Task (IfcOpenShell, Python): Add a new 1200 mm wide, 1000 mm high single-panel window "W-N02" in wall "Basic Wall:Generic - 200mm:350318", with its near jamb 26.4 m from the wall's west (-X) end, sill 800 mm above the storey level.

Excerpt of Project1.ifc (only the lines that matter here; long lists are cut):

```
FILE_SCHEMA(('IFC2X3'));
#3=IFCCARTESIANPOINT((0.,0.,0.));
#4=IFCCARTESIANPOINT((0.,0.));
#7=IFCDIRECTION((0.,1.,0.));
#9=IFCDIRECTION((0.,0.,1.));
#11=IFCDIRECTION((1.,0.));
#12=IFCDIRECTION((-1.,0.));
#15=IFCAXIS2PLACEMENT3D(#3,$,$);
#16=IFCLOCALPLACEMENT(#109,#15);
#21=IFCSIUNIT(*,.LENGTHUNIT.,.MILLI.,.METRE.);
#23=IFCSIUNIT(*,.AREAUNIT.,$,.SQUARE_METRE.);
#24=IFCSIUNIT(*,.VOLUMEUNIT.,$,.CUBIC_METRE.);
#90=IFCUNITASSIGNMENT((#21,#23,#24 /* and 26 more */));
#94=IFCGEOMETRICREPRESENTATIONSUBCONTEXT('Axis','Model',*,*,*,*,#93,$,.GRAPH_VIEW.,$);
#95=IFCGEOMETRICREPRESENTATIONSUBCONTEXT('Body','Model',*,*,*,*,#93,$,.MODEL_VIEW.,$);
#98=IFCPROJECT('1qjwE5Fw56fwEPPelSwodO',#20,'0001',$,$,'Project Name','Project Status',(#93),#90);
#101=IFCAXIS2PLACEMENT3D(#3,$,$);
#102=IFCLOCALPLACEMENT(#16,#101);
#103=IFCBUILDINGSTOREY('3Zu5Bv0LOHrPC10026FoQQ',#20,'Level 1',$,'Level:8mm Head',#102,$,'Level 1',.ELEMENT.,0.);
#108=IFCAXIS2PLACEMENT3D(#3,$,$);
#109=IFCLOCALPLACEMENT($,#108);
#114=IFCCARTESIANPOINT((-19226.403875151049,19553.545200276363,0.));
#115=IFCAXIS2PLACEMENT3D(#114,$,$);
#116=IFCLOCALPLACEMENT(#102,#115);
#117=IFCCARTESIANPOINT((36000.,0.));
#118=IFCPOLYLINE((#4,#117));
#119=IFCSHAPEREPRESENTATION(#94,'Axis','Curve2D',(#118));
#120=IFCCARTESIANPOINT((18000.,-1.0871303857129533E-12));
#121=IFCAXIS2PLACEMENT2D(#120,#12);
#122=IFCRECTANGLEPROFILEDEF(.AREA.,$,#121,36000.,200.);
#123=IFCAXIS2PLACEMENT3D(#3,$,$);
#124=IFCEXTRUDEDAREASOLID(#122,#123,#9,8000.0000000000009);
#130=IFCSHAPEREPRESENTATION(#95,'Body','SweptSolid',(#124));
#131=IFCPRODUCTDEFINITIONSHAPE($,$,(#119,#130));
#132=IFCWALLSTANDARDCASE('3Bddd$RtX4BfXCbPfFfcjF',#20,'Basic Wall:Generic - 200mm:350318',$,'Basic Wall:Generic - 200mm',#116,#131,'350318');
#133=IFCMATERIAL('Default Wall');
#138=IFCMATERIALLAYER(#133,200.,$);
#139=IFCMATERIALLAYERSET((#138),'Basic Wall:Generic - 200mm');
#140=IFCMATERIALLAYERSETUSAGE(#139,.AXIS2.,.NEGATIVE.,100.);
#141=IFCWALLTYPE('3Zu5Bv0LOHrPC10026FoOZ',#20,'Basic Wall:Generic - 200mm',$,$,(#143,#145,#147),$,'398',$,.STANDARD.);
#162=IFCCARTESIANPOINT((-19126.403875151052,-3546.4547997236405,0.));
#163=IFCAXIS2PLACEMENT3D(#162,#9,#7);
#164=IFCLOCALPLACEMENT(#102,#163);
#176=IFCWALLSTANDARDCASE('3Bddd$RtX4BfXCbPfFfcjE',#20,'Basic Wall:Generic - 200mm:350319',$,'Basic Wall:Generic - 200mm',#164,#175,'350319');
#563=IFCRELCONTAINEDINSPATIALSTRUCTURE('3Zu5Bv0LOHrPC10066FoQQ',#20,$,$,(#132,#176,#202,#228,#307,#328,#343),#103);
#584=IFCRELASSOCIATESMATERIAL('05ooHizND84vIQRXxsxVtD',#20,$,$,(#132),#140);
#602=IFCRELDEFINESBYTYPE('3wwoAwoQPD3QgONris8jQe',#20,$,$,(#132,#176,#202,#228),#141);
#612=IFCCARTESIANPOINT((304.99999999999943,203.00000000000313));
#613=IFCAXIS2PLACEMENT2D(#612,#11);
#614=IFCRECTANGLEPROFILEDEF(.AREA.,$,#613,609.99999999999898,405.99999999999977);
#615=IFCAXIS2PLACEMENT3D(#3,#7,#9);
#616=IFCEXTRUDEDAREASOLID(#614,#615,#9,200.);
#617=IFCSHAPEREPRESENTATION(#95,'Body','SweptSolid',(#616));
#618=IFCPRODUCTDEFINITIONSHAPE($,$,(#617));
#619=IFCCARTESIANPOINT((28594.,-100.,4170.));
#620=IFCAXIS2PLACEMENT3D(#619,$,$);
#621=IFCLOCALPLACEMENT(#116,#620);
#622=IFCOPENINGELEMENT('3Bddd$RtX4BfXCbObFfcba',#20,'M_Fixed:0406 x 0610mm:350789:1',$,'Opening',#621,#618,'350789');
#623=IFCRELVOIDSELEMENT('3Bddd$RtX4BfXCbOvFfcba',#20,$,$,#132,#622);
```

```python
import numpy as np
import ifcopenshell
import ifcopenshell.api.feature
import ifcopenshell.api.geometry
import ifcopenshell.api.root
import ifcopenshell.api.spatial
import ifcopenshell.api.type
import ifcopenshell.geom
import ifcopenshell.util.element
import ifcopenshell.util.placement
import ifcopenshell.util.representation
import ifcopenshell.util.shape
import ifcopenshell.util.unit

model = ifcopenshell.open("Project1.ifc")
unit_scale = ifcopenshell.util.unit.calculate_unit_scale(model)
settings = ifcopenshell.geom.settings()


def volume(element):
    """Net volume in cubic metres, openings subtracted."""
    shape = ifcopenshell.geom.create_shape(settings, element)
    return ifcopenshell.util.shape.get_volume(shape.geometry)


wall = model.by_id(132)
storey = ifcopenshell.util.element.get_container(wall, ifc_class="IfcBuildingStorey")
context = ifcopenshell.util.representation.get_context(model, "Model", "Body", "MODEL_VIEW")
before = volume(wall)

width, height, from_end, sill = 1.2, 1, 26.4, 0.8  # metres

# The wall runs along its own X axis, and the end named is its -X end.
wall_shape = ifcopenshell.geom.create_shape(settings, wall)
x, y, z = ifcopenshell.util.shape.get_vertices(wall_shape.geometry).T
start = x.min() + from_end
face, thickness = float(y.min()), float(y.max() - y.min())
wall_matrix = ifcopenshell.util.placement.get_local_placement(wall.ObjectPlacement)
level = ifcopenshell.util.placement.get_local_placement(storey.ObjectPlacement)[2, 3]


def in_wall(x, y):
    """Placement at x, y metres in the wall's axes, at sill height."""
    matrix = wall_matrix.copy()
    matrix[:, 3] = wall_matrix @ np.array([x / unit_scale, y / unit_scale, 0.0, 1.0])
    matrix[2, 3] = level + sill / unit_scale
    return matrix


# Opening: a box that overshoots both wall faces by 50 mm.
opening = ifcopenshell.api.root.create_entity(model, ifc_class="IfcOpeningElement")
box = ifcopenshell.api.geometry.add_wall_representation(
    model, context=context, length=width, height=height, thickness=thickness + 0.1
)
ifcopenshell.api.geometry.assign_representation(model, product=opening, representation=box)
ifcopenshell.api.geometry.edit_object_placement(model, product=opening, matrix=in_wall(start, face - 0.05), is_si=False)
ifcopenshell.api.feature.add_feature(model, feature=opening, element=wall)

window = ifcopenshell.api.root.create_entity(model, ifc_class="IfcWindow", name="W-N02")
window.OverallWidth, window.OverallHeight = width / unit_scale, height / unit_scale
body = ifcopenshell.api.geometry.add_window_representation(
    model,
    context=context,
    overall_width=window.OverallWidth,
    overall_height=window.OverallHeight,
    partition_type="SINGLE_PANEL",
)
ifcopenshell.api.geometry.assign_representation(model, product=window, representation=body)
ifcopenshell.api.spatial.assign_container(model, products=[window], relating_structure=storey)
fills = ifcopenshell.api.feature.add_filling(model, opening=opening, element=window)
fills.OwnerHistory = window.OwnerHistory  # required in IFC2X3

# IFC2X3 keeps the operation on the window style.
style = ifcopenshell.api.root.create_entity(model, ifc_class="IfcWindowStyle", name="W-N02")
style.OperationType, style.ConstructionType = "SINGLE_PANEL", "NOTDEFINED"
style.ParameterTakesPrecedence = style.Sizeable = False
ifcopenshell.api.type.assign_type(model, related_objects=[window], relating_type=style)

# Centre the window in the wall's thickness.
ifcopenshell.api.geometry.edit_object_placement(model, product=window, matrix=in_wall(start, face), is_si=False)
window_shape = ifcopenshell.geom.create_shape(settings, window)
depth = ifcopenshell.util.shape.get_vertices(window_shape.geometry)[:, 1]
offset = face + thickness / 2 - (depth.min() + depth.max()) / 2
ifcopenshell.api.geometry.edit_object_placement(model, product=window, matrix=in_wall(start, offset), is_si=False)

after = volume(wall)

print(f"wall volume {before:.3f} -> {after:.3f} m3")

model.write("Project1_rev.ifc")
```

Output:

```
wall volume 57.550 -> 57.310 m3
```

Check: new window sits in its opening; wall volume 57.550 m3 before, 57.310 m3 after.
